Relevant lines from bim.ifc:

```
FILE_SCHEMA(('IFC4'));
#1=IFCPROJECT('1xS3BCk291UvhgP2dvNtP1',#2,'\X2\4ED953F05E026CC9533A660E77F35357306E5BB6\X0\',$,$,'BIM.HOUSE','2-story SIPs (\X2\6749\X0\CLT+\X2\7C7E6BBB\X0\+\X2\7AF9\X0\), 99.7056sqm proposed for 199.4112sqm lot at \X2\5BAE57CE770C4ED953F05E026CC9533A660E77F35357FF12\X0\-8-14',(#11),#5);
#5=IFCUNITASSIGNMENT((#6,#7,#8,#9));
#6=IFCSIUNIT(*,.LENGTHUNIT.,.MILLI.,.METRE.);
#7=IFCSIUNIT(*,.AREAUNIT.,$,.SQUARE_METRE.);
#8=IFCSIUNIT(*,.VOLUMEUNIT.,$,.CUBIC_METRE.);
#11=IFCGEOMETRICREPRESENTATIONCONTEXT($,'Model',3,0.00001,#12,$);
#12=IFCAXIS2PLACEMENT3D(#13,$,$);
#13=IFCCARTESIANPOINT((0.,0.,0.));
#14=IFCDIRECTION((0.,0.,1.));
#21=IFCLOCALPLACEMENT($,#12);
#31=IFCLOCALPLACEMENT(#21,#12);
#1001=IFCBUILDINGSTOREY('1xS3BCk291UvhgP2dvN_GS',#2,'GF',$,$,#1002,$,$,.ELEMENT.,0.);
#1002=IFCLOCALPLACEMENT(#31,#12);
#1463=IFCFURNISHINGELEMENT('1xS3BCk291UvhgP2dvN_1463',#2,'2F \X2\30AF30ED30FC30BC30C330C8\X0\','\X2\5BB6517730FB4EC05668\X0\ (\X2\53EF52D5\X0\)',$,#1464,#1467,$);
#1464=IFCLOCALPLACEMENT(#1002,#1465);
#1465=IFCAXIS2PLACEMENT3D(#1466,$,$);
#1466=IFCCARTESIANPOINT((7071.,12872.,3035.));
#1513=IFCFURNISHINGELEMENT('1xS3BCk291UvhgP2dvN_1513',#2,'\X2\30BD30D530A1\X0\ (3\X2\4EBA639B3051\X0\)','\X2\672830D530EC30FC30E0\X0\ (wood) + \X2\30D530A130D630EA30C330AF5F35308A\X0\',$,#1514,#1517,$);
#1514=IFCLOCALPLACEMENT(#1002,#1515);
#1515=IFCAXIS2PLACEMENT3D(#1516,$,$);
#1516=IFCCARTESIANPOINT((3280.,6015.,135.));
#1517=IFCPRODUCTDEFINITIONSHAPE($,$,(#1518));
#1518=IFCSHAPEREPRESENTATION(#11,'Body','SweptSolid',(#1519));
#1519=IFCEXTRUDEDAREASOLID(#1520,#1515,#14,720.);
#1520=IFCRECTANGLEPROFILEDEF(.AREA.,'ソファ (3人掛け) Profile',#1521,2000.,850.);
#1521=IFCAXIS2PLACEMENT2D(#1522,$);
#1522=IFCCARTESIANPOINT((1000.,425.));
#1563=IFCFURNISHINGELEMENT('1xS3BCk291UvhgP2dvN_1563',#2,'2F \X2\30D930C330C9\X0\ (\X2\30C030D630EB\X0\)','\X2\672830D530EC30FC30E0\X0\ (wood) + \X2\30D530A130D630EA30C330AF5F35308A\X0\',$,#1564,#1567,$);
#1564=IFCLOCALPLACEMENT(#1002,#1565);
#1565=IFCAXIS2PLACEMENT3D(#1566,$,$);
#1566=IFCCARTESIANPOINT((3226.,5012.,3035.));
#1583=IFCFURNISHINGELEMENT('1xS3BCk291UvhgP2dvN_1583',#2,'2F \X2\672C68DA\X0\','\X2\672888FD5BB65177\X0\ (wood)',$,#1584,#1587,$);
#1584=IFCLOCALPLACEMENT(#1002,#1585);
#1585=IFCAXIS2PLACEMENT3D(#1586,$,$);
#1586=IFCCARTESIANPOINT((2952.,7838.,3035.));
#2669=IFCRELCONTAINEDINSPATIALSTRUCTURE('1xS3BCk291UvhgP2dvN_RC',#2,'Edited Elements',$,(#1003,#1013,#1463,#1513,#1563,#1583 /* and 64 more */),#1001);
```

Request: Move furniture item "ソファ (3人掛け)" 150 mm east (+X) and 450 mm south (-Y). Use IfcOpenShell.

```python
import ifcopenshell
import ifcopenshell.api.geometry
import ifcopenshell.util.placement
import ifcopenshell.util.unit

model = ifcopenshell.open("bim.ifc")
unit_scale = ifcopenshell.util.unit.calculate_unit_scale(model)

item = model.by_guid("1xS3BCk291UvhgP2dvN_1513")
matrix = ifcopenshell.util.placement.get_local_placement(item.ObjectPlacement)
matrix[0, 3] += 0.15 / unit_scale
matrix[1, 3] -= 0.45 / unit_scale
ifcopenshell.api.geometry.edit_object_placement(model, product=item, matrix=matrix, is_si=False)

print(ifcopenshell.util.placement.get_local_placement(item.ObjectPlacement).round(3) + 0.0)

model.write("bim_rev.ifc")
```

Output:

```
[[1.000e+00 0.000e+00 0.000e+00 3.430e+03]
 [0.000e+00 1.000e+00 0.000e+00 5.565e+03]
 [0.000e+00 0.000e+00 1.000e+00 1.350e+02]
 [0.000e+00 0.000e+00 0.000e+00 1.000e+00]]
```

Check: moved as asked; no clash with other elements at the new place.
